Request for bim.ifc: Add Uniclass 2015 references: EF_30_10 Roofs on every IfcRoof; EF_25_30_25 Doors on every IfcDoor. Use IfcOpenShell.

First a look at what the model holds.

```python
import ifcopenshell

model = ifcopenshell.open("bim.ifc")
print(model.schema)
print("classifications:", [c.Name for c in model.by_type("IfcClassification")])
for ifc_class in ("IfcDoor", "IfcRoof", "IfcStair", "IfcWall", "IfcWindow"):
    print(ifc_class, len(model.by_type(ifc_class)))
```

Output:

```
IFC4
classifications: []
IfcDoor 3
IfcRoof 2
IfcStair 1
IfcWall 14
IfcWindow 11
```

```python
import ifcopenshell
import ifcopenshell.api.classification

model = ifcopenshell.open("bim.ifc")

system = ifcopenshell.api.classification.add_classification(model, classification="Uniclass 2015")

codes = {
    "IfcRoof": ("EF_30_10", "Roofs"),
    "IfcDoor": ("EF_25_30_25", "Doors"),
}
for ifc_class, (code, name) in codes.items():
    products = model.by_type(ifc_class)
    ifcopenshell.api.classification.add_reference(
        model, products=products, classification=system, identification=code, name=name
    )
    print(code, len(products))

model.write("bim-out.ifc")
```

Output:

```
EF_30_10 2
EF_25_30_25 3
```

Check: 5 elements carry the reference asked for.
